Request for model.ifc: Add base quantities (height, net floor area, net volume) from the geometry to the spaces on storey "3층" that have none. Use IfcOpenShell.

First a look at what the model holds.

```python
import ifcopenshell
import ifcopenshell.util.element
import ifcopenshell.util.unit

model = ifcopenshell.open("model.ifc")
print(model.schema)
for unit_type in ("LENGTHUNIT", "AREAUNIT", "VOLUMEUNIT"):
    print(unit_type, ifcopenshell.util.unit.calculate_unit_scale(model, unit_type))
storey = next(s for s in model.by_type("IfcBuildingStorey") if s.Name == "3층")
spaces = [e for e in ifcopenshell.util.element.get_decomposition(storey) if e.is_a("IfcSpace")]
for e in sorted(spaces, key=lambda e: e.id()):
    print(e.id(), e.is_a(), e.Name, list(ifcopenshell.util.element.get_psets(e, qtos_only=True)), sep=" | ")
```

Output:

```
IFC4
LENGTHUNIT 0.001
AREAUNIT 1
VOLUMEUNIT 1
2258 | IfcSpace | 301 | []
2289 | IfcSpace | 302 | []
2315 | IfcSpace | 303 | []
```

```python
import ifcopenshell
import ifcopenshell.api.pset
import ifcopenshell.geom
import ifcopenshell.util.element
import ifcopenshell.util.shape
import ifcopenshell.util.unit

model = ifcopenshell.open("model.ifc")
unit_scale = ifcopenshell.util.unit.calculate_unit_scale(model)
area_scale = ifcopenshell.util.unit.calculate_unit_scale(model, "AREAUNIT")
volume_scale = ifcopenshell.util.unit.calculate_unit_scale(model, "VOLUMEUNIT")
settings = ifcopenshell.geom.settings()

storey = next(s for s in model.by_type("IfcBuildingStorey") if s.Name == "3층")
spaces = [e for e in ifcopenshell.util.element.get_decomposition(storey) if e.is_a("IfcSpace")]

for e in sorted(spaces, key=lambda e: e.id()):
    if ifcopenshell.util.element.get_psets(e, qtos_only=True, should_inherit=False):
        continue
    # Geometry comes back in metres, in the element's own axes.
    shape = ifcopenshell.geom.create_shape(settings, e)
    values = {
        "Height": ifcopenshell.util.shape.get_z(shape.geometry) / unit_scale,
        "NetFloorArea": ifcopenshell.util.shape.get_footprint_area(shape.geometry) / area_scale,
        "NetVolume": ifcopenshell.util.shape.get_volume(shape.geometry) / volume_scale,
    }
    qto = ifcopenshell.api.pset.add_qto(model, product=e, name="Qto_SpaceBaseQuantities")
    ifcopenshell.api.pset.edit_qto(model, qto=qto, properties=values)
    print(e.id(), {k: round(v, 3) for k, v in values.items()})

model.write("model_updated.ifc")
```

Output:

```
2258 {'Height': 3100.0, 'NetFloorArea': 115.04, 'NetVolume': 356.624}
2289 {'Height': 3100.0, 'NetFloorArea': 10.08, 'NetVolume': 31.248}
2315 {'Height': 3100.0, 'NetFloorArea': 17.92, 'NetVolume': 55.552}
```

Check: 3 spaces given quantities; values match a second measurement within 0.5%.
